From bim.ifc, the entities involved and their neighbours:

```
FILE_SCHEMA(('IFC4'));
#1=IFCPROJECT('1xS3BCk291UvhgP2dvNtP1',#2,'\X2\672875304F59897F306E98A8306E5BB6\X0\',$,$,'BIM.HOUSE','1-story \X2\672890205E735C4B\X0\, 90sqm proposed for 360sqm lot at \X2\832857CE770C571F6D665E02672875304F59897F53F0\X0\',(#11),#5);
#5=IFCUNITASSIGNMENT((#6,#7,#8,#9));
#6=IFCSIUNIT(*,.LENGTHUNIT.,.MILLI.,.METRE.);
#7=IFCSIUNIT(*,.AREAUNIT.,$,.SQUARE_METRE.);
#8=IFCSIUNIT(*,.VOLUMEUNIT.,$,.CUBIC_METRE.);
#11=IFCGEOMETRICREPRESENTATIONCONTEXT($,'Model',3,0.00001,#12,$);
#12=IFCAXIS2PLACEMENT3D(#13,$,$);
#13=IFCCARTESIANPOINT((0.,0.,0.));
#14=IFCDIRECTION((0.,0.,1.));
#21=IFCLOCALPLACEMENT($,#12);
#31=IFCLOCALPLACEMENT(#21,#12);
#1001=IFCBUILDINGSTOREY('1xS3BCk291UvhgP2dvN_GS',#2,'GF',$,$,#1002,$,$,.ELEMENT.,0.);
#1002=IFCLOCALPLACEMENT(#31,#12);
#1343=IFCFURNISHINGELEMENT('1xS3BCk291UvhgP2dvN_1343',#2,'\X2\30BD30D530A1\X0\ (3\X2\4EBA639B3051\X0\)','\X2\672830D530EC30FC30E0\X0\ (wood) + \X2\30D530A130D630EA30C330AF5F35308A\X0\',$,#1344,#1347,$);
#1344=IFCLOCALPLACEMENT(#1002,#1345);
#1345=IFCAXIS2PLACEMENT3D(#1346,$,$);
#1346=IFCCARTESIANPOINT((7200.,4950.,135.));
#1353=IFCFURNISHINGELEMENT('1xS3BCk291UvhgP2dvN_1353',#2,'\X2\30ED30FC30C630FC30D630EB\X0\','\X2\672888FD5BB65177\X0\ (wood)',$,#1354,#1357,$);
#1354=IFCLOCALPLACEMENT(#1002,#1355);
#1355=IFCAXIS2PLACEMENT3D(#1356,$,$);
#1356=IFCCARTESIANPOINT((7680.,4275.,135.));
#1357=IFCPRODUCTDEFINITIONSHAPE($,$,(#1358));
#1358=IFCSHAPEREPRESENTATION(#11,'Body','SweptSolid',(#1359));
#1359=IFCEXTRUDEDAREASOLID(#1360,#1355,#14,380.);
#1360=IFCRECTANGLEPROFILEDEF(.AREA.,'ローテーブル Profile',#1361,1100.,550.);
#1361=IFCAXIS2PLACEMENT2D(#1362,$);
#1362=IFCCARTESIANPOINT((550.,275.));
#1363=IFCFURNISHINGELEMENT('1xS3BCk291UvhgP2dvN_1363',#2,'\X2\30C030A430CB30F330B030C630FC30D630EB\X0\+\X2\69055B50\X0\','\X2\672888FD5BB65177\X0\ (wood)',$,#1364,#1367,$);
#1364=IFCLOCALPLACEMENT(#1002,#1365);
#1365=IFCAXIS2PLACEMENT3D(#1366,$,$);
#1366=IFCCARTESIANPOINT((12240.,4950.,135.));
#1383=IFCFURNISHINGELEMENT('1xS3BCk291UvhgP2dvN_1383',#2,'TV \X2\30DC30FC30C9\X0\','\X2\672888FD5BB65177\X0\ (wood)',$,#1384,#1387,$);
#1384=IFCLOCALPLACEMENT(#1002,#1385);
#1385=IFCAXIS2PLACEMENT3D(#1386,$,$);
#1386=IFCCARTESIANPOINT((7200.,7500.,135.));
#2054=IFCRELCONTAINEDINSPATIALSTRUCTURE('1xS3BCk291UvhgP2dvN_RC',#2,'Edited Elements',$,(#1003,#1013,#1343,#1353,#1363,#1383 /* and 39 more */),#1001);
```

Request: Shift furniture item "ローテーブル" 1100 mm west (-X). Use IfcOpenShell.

```python
import ifcopenshell
import ifcopenshell.api.geometry
import ifcopenshell.util.placement

model = ifcopenshell.open("bim.ifc")

item = model.by_guid("1xS3BCk291UvhgP2dvN_1353")
matrix = ifcopenshell.util.placement.get_local_placement(item.ObjectPlacement)
matrix[0, 3] -= 1100.0
ifcopenshell.api.geometry.edit_object_placement(model, product=item, matrix=matrix, is_si=False)

print(ifcopenshell.util.placement.get_local_placement(item.ObjectPlacement).round(3) + 0.0)

model.write("bim-out.ifc")
```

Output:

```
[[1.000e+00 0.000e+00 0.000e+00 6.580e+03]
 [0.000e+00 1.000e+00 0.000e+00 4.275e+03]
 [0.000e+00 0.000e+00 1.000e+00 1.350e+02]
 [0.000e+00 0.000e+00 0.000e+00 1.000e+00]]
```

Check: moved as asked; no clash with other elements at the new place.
